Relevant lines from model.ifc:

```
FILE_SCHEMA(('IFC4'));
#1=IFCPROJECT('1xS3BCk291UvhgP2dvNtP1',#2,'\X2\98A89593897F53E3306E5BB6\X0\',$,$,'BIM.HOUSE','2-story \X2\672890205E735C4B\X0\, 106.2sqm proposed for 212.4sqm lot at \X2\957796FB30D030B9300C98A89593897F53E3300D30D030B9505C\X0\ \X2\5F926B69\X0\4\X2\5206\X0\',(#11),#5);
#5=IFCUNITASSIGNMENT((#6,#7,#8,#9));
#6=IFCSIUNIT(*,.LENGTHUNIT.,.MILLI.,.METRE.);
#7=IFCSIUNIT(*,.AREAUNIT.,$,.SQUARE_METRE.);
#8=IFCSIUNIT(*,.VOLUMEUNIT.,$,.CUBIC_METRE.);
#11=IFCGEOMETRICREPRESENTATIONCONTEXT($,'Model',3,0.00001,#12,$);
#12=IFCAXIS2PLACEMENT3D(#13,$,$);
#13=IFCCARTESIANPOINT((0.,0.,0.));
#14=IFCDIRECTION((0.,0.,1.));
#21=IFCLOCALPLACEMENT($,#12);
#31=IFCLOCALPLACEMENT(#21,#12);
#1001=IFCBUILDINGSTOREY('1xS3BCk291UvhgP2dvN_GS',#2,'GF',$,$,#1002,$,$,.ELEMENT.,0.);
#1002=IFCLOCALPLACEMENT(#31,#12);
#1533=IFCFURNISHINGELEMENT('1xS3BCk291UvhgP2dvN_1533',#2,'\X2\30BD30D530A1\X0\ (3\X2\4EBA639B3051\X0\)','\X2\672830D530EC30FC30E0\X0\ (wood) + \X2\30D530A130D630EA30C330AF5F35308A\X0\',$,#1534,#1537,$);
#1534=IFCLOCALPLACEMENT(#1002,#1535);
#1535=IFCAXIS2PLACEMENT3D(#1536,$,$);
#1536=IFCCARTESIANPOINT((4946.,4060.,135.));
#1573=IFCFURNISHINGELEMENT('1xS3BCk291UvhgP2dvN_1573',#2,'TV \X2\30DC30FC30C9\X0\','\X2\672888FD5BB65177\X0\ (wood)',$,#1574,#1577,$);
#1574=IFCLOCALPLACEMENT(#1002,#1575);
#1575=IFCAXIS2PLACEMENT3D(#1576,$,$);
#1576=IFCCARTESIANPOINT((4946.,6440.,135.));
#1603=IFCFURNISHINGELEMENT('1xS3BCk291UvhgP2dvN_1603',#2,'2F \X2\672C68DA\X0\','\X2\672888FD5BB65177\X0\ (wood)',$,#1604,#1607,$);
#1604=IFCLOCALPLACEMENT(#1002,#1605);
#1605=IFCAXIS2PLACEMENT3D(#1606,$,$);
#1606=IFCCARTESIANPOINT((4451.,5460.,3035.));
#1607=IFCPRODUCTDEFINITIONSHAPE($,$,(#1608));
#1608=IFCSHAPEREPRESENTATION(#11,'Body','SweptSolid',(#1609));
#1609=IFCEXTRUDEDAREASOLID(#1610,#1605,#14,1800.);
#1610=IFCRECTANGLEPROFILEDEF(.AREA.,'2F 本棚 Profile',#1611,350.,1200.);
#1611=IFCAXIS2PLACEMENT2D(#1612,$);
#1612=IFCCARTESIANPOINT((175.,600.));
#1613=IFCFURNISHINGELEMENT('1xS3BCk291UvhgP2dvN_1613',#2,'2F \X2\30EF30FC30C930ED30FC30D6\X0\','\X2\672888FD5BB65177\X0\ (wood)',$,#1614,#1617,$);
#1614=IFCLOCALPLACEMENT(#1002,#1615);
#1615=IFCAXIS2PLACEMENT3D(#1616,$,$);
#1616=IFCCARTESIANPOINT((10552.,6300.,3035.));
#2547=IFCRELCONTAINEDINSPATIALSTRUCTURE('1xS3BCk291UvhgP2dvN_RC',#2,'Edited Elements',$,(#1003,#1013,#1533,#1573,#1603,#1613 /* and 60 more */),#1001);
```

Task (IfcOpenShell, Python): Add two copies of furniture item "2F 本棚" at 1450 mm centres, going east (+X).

```python
import numpy as np
import ifcopenshell
import ifcopenshell.api.geometry
import ifcopenshell.api.root
import ifcopenshell.util.element
import ifcopenshell.util.placement
import ifcopenshell.util.unit

model = ifcopenshell.open("model.ifc")
unit_scale = ifcopenshell.util.unit.calculate_unit_scale(model)


def reuse_history(source, copy):
    """copy_class also copies each property set's owner history, people and application; keep the originals."""
    for rel in copy.IsDefinedBy:
        if rel.is_a("IfcRelDefinesByProperties") and (history := rel.RelatingPropertyDefinition.OwnerHistory):
            rel.RelatingPropertyDefinition.OwnerHistory = source.OwnerHistory
            ifcopenshell.util.element.remove_deep2(model, history)


source = model.by_id(1603)
base = ifcopenshell.util.placement.get_local_placement(source.ObjectPlacement)
step = np.array([1.0, 0.0, 0.0]) * 1.45 / unit_scale

for i in range(1, 3):
    copy = ifcopenshell.api.root.copy_class(model, product=source)
    copy.Representation = ifcopenshell.util.element.copy_deep(
        model, source.Representation, exclude=["IfcGeometricRepresentationContext", "IfcRepresentationMap"]
    )
    reuse_history(source, copy)
    matrix = base.copy()
    matrix[:3, 3] += i * step
    print("added at", matrix[:3, 3].round(3) + 0.0)
    ifcopenshell.api.geometry.edit_object_placement(model, product=copy, matrix=matrix, is_si=False)

model.write("model_v2.ifc")
```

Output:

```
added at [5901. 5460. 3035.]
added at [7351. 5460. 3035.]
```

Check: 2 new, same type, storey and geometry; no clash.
